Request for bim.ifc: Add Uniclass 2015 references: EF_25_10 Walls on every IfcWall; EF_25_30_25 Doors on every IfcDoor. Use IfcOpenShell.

First a look at what the model holds.

```python
import ifcopenshell

model = ifcopenshell.open("bim.ifc")
print(model.schema)
print("classifications:", [c.Name for c in model.by_type("IfcClassification")])
for ifc_class in ("IfcDoor", "IfcRoof", "IfcStair", "IfcWall", "IfcWindow"):
    print(ifc_class, len(model.by_type(ifc_class)))
```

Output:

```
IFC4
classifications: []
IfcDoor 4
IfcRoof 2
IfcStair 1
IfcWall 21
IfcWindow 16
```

```python
import ifcopenshell
import ifcopenshell.api.classification

model = ifcopenshell.open("bim.ifc")

system = ifcopenshell.api.classification.add_classification(model, classification="Uniclass 2015")

codes = {
    "IfcWall": ("EF_25_10", "Walls"),
    "IfcDoor": ("EF_25_30_25", "Doors"),
}
for ifc_class, (code, name) in codes.items():
    products = model.by_type(ifc_class)
    ifcopenshell.api.classification.add_reference(
        model, products=products, classification=system, identification=code, name=name
    )
    print(code, len(products))

model.write("bim_updated.ifc")
```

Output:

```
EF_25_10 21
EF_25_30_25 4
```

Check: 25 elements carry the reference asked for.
